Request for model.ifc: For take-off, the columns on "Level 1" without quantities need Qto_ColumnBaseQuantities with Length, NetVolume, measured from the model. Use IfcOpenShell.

First a look at what the model holds.

```python
import ifcopenshell
import ifcopenshell.util.element
import ifcopenshell.util.unit

model = ifcopenshell.open("model.ifc")
print(model.schema)
for unit_type in ("LENGTHUNIT", "AREAUNIT", "VOLUMEUNIT"):
    print(unit_type, ifcopenshell.util.unit.calculate_unit_scale(model, unit_type))
storey = next(s for s in model.by_type("IfcBuildingStorey") if s.Name == "Level 1")
columns = [e for e in ifcopenshell.util.element.get_decomposition(storey) if e.is_a("IfcColumn")]
for e in sorted(columns, key=lambda e: e.id()):
    print(e.id(), e.is_a(), e.Name, list(ifcopenshell.util.element.get_psets(e, qtos_only=True)), sep=" | ")
```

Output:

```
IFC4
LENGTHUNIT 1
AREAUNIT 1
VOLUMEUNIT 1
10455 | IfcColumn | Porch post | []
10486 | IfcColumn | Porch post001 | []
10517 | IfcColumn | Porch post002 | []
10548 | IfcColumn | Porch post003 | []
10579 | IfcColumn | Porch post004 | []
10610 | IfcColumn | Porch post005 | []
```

```python
import ifcopenshell
import ifcopenshell.api.pset
import ifcopenshell.geom
import ifcopenshell.util.element
import ifcopenshell.util.shape
import ifcopenshell.util.unit

model = ifcopenshell.open("model.ifc")
unit_scale = ifcopenshell.util.unit.calculate_unit_scale(model)
volume_scale = ifcopenshell.util.unit.calculate_unit_scale(model, "VOLUMEUNIT")
settings = ifcopenshell.geom.settings()

storey = next(s for s in model.by_type("IfcBuildingStorey") if s.Name == "Level 1")
columns = [e for e in ifcopenshell.util.element.get_decomposition(storey) if e.is_a("IfcColumn")]

for e in sorted(columns, key=lambda e: e.id()):
    if ifcopenshell.util.element.get_psets(e, qtos_only=True, should_inherit=False):
        continue
    # Geometry comes back in metres, in the element's own axes.
    shape = ifcopenshell.geom.create_shape(settings, e)
    values = {
        "Length": ifcopenshell.util.shape.get_z(shape.geometry) / unit_scale,
        "NetVolume": ifcopenshell.util.shape.get_volume(shape.geometry) / volume_scale,
    }
    qto = ifcopenshell.api.pset.add_qto(model, product=e, name="Qto_ColumnBaseQuantities")
    ifcopenshell.api.pset.edit_qto(model, qto=qto, properties=values)
    print(e.id(), {k: round(v, 3) for k, v in values.items()})

model.write("model_edited.ifc")
```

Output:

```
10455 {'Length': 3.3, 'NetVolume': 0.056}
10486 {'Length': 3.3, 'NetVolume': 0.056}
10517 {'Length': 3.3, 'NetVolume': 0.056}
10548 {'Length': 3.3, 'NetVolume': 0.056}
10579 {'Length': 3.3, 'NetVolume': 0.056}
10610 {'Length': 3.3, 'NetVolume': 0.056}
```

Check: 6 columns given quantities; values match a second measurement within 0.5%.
